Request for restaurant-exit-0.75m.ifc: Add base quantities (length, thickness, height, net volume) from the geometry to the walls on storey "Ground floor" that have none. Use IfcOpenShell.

First a look at what the model holds.

```python
import ifcopenshell
import ifcopenshell.util.element
import ifcopenshell.util.unit

model = ifcopenshell.open("restaurant-exit-0.75m.ifc")
print(model.schema)
for unit_type in ("LENGTHUNIT", "AREAUNIT", "VOLUMEUNIT"):
    print(unit_type, ifcopenshell.util.unit.calculate_unit_scale(model, unit_type))
storey = next(s for s in model.by_type("IfcBuildingStorey") if s.Name == "Ground floor")
walls = [e for e in ifcopenshell.util.element.get_decomposition(storey) if e.is_a("IfcWall")]
for e in sorted(walls, key=lambda e: e.id()):
    print(e.id(), e.is_a(), e.Name, list(ifcopenshell.util.element.get_psets(e, qtos_only=True)), sep=" | ")
```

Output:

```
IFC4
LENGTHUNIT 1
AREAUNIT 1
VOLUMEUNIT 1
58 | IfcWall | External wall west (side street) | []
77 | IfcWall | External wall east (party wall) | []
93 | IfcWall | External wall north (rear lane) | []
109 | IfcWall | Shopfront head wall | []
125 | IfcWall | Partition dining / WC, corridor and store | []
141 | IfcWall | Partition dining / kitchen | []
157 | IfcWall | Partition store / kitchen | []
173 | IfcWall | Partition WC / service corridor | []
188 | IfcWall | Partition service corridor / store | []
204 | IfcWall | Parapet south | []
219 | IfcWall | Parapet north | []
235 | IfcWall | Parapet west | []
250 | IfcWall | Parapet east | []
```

```python
import ifcopenshell
import ifcopenshell.api.pset
import ifcopenshell.geom
import ifcopenshell.util.element
import ifcopenshell.util.shape
import ifcopenshell.util.unit

model = ifcopenshell.open("restaurant-exit-0.75m.ifc")
unit_scale = ifcopenshell.util.unit.calculate_unit_scale(model)
volume_scale = ifcopenshell.util.unit.calculate_unit_scale(model, "VOLUMEUNIT")
settings = ifcopenshell.geom.settings()

storey = next(s for s in model.by_type("IfcBuildingStorey") if s.Name == "Ground floor")
walls = [e for e in ifcopenshell.util.element.get_decomposition(storey) if e.is_a("IfcWall")]

for e in sorted(walls, key=lambda e: e.id()):
    if ifcopenshell.util.element.get_psets(e, qtos_only=True, should_inherit=False):
        continue
    # Geometry comes back in metres, in the element's own axes.
    shape = ifcopenshell.geom.create_shape(settings, e)
    values = {
        "Length": ifcopenshell.util.shape.get_x(shape.geometry) / unit_scale,
        "Width": ifcopenshell.util.shape.get_y(shape.geometry) / unit_scale,
        "Height": ifcopenshell.util.shape.get_z(shape.geometry) / unit_scale,
        "NetVolume": ifcopenshell.util.shape.get_volume(shape.geometry) / volume_scale,
    }
    qto = ifcopenshell.api.pset.add_qto(model, product=e, name="Qto_WallBaseQuantities")
    ifcopenshell.api.pset.edit_qto(model, qto=qto, properties=values)
    print(e.id(), {k: round(v, 3) for k, v in values.items()})

model.write("restaurant-exit-0.75m_edited.ifc")
```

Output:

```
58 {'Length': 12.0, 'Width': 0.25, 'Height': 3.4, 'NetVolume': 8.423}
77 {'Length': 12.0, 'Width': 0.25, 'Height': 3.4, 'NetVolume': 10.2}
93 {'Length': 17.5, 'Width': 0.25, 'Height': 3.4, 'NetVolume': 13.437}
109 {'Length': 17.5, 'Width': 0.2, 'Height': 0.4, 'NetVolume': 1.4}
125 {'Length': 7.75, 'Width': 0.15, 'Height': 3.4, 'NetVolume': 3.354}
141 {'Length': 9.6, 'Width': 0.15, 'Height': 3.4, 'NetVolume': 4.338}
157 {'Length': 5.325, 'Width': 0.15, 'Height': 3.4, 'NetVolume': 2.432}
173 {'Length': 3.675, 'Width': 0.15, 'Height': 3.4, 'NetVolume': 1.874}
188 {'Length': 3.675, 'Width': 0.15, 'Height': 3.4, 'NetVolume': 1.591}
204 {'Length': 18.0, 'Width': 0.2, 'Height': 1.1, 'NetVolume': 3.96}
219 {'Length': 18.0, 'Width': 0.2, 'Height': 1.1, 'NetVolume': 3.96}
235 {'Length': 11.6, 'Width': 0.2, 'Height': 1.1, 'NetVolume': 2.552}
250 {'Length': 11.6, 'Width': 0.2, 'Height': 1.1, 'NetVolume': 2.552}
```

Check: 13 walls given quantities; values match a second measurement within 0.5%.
